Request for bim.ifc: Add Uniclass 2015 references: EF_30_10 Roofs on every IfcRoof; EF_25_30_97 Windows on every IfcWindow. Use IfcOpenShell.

First a look at what the model holds.

```python
import ifcopenshell

model = ifcopenshell.open("bim.ifc")
print(model.schema)
print("classifications:", [c.Name for c in model.by_type("IfcClassification")])
for ifc_class in ("IfcDoor", "IfcRoof", "IfcStair", "IfcWall", "IfcWindow"):
    print(ifc_class, len(model.by_type(ifc_class)))
```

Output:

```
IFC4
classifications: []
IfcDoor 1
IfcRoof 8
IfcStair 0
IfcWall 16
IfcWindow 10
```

```python
import ifcopenshell
import ifcopenshell.api.classification

model = ifcopenshell.open("bim.ifc")

system = ifcopenshell.api.classification.add_classification(model, classification="Uniclass 2015")

codes = {
    "IfcRoof": ("EF_30_10", "Roofs"),
    "IfcWindow": ("EF_25_30_97", "Windows"),
}
for ifc_class, (code, name) in codes.items():
    products = model.by_type(ifc_class)
    ifcopenshell.api.classification.add_reference(
        model, products=products, classification=system, identification=code, name=name
    )
    print(code, len(products))

model.write("bim_rev.ifc")
```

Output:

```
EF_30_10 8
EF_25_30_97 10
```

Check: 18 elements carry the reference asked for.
